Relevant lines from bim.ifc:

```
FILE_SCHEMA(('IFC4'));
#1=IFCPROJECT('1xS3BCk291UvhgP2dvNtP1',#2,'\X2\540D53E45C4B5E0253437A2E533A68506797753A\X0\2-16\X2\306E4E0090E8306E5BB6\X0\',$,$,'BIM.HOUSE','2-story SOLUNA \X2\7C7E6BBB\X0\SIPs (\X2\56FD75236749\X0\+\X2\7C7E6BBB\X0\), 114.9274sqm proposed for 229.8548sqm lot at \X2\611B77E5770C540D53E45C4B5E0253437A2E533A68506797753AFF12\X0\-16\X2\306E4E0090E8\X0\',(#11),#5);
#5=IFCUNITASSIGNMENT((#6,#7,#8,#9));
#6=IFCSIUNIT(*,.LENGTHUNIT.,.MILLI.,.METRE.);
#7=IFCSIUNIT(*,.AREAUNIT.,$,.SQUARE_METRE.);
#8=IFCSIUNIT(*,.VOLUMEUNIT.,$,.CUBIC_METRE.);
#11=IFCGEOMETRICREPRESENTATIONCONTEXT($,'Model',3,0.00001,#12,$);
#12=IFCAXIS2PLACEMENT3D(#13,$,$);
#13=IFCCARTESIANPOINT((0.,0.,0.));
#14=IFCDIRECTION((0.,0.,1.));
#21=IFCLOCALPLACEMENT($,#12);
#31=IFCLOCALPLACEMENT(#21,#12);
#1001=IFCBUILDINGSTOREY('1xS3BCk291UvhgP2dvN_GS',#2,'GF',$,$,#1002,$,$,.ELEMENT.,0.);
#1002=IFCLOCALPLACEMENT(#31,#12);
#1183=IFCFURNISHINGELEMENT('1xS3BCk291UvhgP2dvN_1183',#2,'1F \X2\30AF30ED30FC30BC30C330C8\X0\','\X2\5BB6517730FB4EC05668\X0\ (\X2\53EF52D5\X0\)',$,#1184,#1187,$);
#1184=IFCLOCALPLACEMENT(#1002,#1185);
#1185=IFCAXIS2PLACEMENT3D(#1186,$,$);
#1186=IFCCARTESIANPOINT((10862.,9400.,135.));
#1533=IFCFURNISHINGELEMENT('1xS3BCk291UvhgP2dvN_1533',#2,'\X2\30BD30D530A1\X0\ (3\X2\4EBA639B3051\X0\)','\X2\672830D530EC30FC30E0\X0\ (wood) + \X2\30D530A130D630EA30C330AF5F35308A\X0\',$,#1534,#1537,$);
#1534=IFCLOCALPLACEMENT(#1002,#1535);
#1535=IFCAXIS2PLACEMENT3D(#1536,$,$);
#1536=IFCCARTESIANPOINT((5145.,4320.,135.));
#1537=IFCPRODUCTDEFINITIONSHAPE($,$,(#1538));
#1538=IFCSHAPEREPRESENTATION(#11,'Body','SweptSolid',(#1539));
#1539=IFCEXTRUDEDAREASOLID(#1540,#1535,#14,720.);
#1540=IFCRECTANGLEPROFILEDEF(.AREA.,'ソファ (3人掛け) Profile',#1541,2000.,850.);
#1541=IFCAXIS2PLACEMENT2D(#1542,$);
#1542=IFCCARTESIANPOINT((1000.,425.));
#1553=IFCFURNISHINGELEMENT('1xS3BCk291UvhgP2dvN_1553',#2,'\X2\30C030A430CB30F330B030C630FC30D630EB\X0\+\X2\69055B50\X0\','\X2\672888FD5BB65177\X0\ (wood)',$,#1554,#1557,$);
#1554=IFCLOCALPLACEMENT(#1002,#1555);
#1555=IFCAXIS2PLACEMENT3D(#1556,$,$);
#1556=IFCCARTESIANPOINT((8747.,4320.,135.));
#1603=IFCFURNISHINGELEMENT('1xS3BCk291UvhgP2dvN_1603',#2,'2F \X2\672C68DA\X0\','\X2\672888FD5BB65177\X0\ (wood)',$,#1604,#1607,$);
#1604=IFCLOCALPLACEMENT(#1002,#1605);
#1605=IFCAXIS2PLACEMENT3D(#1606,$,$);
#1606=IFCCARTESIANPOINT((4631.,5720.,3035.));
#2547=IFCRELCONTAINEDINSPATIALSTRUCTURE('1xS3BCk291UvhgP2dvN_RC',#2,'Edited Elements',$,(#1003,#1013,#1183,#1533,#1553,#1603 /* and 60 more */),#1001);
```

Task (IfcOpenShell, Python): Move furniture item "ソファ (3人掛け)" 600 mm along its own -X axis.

```python
import ifcopenshell
import ifcopenshell.api.geometry
import ifcopenshell.util.placement
import ifcopenshell.util.unit

model = ifcopenshell.open("bim.ifc")
unit_scale = ifcopenshell.util.unit.calculate_unit_scale(model)

item = model.by_guid("1xS3BCk291UvhgP2dvN_1533")
matrix = ifcopenshell.util.placement.get_local_placement(item.ObjectPlacement)
matrix[:3, 3] -= matrix[:3, 0] * 0.6 / unit_scale
ifcopenshell.api.geometry.edit_object_placement(model, product=item, matrix=matrix, is_si=False)

print(ifcopenshell.util.placement.get_local_placement(item.ObjectPlacement).round(3) + 0.0)

model.write("bim_v2.ifc")
```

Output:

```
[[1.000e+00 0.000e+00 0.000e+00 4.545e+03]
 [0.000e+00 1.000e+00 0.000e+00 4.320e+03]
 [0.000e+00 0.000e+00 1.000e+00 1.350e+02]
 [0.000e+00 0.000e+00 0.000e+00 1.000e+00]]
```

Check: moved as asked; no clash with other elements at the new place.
